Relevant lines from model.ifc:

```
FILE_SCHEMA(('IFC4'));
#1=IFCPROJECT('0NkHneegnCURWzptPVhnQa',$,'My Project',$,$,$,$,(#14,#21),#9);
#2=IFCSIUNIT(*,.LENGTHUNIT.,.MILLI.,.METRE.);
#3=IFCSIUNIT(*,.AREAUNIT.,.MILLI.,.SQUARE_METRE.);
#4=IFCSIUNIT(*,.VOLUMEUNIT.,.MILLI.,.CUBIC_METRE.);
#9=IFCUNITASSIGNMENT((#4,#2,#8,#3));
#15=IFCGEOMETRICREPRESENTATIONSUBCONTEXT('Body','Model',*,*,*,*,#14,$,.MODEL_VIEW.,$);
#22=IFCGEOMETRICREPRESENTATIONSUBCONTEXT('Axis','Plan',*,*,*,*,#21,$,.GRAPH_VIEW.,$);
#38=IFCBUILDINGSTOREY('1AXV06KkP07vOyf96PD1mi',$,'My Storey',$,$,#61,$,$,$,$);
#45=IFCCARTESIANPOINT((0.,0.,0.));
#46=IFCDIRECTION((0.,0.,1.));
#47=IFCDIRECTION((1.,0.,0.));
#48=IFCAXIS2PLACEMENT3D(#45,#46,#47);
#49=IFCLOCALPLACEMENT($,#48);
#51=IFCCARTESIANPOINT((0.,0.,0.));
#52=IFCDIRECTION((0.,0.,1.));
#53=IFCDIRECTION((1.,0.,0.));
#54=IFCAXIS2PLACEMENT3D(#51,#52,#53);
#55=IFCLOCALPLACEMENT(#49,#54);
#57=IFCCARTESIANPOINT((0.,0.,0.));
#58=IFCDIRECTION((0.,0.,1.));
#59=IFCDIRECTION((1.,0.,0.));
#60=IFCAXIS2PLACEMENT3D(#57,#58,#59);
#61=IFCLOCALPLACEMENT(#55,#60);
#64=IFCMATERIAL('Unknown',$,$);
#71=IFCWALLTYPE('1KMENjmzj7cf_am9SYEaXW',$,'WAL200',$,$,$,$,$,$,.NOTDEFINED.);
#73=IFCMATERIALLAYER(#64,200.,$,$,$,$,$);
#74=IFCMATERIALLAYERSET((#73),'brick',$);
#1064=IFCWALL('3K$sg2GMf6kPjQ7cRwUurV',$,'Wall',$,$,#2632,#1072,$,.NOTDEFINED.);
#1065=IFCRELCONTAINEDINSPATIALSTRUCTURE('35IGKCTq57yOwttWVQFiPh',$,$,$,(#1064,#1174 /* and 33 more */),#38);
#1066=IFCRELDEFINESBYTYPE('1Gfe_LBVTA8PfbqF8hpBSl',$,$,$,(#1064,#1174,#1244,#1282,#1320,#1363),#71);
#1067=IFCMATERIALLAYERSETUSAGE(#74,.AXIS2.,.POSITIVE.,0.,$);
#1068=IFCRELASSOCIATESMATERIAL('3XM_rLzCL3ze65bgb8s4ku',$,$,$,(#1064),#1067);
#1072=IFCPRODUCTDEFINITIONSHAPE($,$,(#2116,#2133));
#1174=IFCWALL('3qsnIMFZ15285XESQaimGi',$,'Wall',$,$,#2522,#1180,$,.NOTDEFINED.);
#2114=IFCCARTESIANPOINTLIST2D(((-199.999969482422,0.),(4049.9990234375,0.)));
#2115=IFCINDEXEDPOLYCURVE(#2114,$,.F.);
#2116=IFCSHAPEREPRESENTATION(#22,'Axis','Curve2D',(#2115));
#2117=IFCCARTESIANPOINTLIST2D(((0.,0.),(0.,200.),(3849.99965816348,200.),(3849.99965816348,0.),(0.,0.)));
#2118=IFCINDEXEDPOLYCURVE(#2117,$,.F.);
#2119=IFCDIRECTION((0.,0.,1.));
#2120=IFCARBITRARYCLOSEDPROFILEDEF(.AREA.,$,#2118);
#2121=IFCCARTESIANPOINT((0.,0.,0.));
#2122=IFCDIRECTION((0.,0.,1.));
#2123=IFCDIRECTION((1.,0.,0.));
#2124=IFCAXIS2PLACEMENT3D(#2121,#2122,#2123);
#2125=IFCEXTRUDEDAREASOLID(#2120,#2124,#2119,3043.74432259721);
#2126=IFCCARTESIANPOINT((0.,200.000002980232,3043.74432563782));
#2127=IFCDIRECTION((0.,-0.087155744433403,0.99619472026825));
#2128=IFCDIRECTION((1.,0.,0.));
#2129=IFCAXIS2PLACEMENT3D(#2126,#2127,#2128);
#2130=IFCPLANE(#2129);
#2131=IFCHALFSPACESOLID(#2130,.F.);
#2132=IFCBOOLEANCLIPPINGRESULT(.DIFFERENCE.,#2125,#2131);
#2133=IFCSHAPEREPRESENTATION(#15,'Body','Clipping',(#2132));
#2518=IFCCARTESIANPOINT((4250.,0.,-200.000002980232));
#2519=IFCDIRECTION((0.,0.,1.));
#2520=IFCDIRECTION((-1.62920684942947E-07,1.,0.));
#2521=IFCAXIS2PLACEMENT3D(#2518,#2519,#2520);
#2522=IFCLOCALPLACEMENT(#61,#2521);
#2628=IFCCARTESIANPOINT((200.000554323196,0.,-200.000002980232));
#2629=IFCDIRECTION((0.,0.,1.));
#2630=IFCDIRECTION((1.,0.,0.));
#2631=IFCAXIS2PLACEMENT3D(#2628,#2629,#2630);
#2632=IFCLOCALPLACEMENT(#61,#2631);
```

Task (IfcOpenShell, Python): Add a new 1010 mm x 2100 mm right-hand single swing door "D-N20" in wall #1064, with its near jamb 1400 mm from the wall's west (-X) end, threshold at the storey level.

```python
import numpy as np
import ifcopenshell
import ifcopenshell.api.feature
import ifcopenshell.api.geometry
import ifcopenshell.api.root
import ifcopenshell.api.spatial
import ifcopenshell.geom
import ifcopenshell.util.element
import ifcopenshell.util.placement
import ifcopenshell.util.representation
import ifcopenshell.util.shape
import ifcopenshell.util.unit

model = ifcopenshell.open("model.ifc")
unit_scale = ifcopenshell.util.unit.calculate_unit_scale(model)
settings = ifcopenshell.geom.settings()


def volume(element):
    """Net volume in cubic metres, openings subtracted."""
    shape = ifcopenshell.geom.create_shape(settings, element)
    return ifcopenshell.util.shape.get_volume(shape.geometry)


wall = model.by_guid("3K$sg2GMf6kPjQ7cRwUurV")
storey = ifcopenshell.util.element.get_container(wall, ifc_class="IfcBuildingStorey")
context = ifcopenshell.util.representation.get_context(model, "Model", "Body", "MODEL_VIEW")
before = volume(wall)

width, height, from_end, sill = 1.01, 2.1, 1.4, 0.0  # metres

# The wall runs along its own X axis, and the end named is its -X end.
wall_shape = ifcopenshell.geom.create_shape(settings, wall)
x, y, z = ifcopenshell.util.shape.get_vertices(wall_shape.geometry).T
start = x.min() + from_end
face, thickness = float(y.min()), float(y.max() - y.min())
wall_matrix = ifcopenshell.util.placement.get_local_placement(wall.ObjectPlacement)
level = ifcopenshell.util.placement.get_local_placement(storey.ObjectPlacement)[2, 3]


def in_wall(x, y):
    """Placement at x, y metres in the wall's axes, at sill height."""
    matrix = wall_matrix.copy()
    matrix[:, 3] = wall_matrix @ np.array([x / unit_scale, y / unit_scale, 0.0, 1.0])
    matrix[2, 3] = level + sill / unit_scale
    return matrix


# Opening: a box that overshoots both wall faces by 50 mm.
opening = ifcopenshell.api.root.create_entity(model, ifc_class="IfcOpeningElement", predefined_type="OPENING")
box = ifcopenshell.api.geometry.add_wall_representation(
    model, context=context, length=width, height=height, thickness=thickness + 0.1
)
ifcopenshell.api.geometry.assign_representation(model, product=opening, representation=box)
ifcopenshell.api.geometry.edit_object_placement(model, product=opening, matrix=in_wall(start, face - 0.05), is_si=False)
ifcopenshell.api.feature.add_feature(model, feature=opening, element=wall)

door = ifcopenshell.api.root.create_entity(model, ifc_class="IfcDoor", name="D-N20", predefined_type="DOOR")
door.OverallWidth, door.OverallHeight = width / unit_scale, height / unit_scale
door.OperationType = "SINGLE_SWING_RIGHT"
body = ifcopenshell.api.geometry.add_door_representation(
    model,
    context=context,
    overall_width=door.OverallWidth,
    overall_height=door.OverallHeight,
    operation_type="SINGLE_SWING_RIGHT",
    lining_properties={"LiningDepth": thickness / unit_scale, "ThresholdDepth": thickness / unit_scale},
)
ifcopenshell.api.geometry.assign_representation(model, product=door, representation=body)
ifcopenshell.api.spatial.assign_container(model, products=[door], relating_structure=storey)
ifcopenshell.api.feature.add_filling(model, opening=opening, element=door)

# The lining spans the wall, so the door starts at the wall face.
ifcopenshell.api.geometry.edit_object_placement(model, product=door, matrix=in_wall(start, face), is_si=False)

after = volume(wall)

print(f"wall volume {before:.3f} -> {after:.3f} m3")

model.write("model_edited.ifc")
```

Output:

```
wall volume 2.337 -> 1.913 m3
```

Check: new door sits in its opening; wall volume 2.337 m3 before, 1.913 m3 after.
